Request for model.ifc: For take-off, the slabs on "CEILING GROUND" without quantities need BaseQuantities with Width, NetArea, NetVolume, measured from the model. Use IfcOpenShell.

First a look at what the model holds.

```python
import ifcopenshell
import ifcopenshell.util.element
import ifcopenshell.util.unit

model = ifcopenshell.open("model.ifc")
print(model.schema)
for unit_type in ("LENGTHUNIT", "AREAUNIT", "VOLUMEUNIT"):
    print(unit_type, ifcopenshell.util.unit.calculate_unit_scale(model, unit_type))
storey = next(s for s in model.by_type("IfcBuildingStorey") if s.Name == "CEILING GROUND")
slabs = [e for e in ifcopenshell.util.element.get_decomposition(storey) if e.is_a("IfcSlab")]
for e in sorted(slabs, key=lambda e: e.id()):
    print(e.id(), e.is_a(), e.Name, list(ifcopenshell.util.element.get_psets(e, qtos_only=True)), sep=" | ")
```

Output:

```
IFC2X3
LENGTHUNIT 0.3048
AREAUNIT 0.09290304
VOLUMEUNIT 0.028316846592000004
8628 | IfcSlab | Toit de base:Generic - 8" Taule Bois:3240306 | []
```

```python
import ifcopenshell
import ifcopenshell.api.pset
import ifcopenshell.geom
import ifcopenshell.util.element
import ifcopenshell.util.shape
import ifcopenshell.util.unit

model = ifcopenshell.open("model.ifc")
unit_scale = ifcopenshell.util.unit.calculate_unit_scale(model)
area_scale = ifcopenshell.util.unit.calculate_unit_scale(model, "AREAUNIT")
volume_scale = ifcopenshell.util.unit.calculate_unit_scale(model, "VOLUMEUNIT")
settings = ifcopenshell.geom.settings()

storey = next(s for s in model.by_type("IfcBuildingStorey") if s.Name == "CEILING GROUND")
slabs = [e for e in ifcopenshell.util.element.get_decomposition(storey) if e.is_a("IfcSlab")]

for e in sorted(slabs, key=lambda e: e.id()):
    if ifcopenshell.util.element.get_psets(e, qtos_only=True, should_inherit=False):
        continue
    # Geometry comes back in metres, in the element's own axes.
    shape = ifcopenshell.geom.create_shape(settings, e)
    values = {
        "Width": ifcopenshell.util.shape.get_z(shape.geometry) / unit_scale,
        "NetArea": ifcopenshell.util.shape.get_footprint_area(shape.geometry) / area_scale,
        "NetVolume": ifcopenshell.util.shape.get_volume(shape.geometry) / volume_scale,
    }
    qto = ifcopenshell.api.pset.add_qto(model, product=e, name="BaseQuantities")
    ifcopenshell.api.pset.edit_qto(model, qto=qto, properties=values)
    print(e.id(), {k: round(v, 3) for k, v in values.items()})

model.write("model_edited.ifc")
```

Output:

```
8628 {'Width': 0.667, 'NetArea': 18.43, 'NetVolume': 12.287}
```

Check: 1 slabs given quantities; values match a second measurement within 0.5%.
